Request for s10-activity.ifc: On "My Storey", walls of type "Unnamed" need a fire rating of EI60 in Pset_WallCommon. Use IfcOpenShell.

First a look at what the model holds.

```python
import ifcopenshell
import ifcopenshell.util.element

model = ifcopenshell.open("s10-activity.ifc")
print(model.schema)
storey = next(s for s in model.by_type("IfcBuildingStorey") if s.Name == "My Storey")
walls = [e for e in ifcopenshell.util.element.get_decomposition(storey) if e.is_a("IfcWall")]
seen = {}
for e in walls:
    element_type = ifcopenshell.util.element.get_type(e)
    key = (element_type.Name if element_type != e and element_type else None, ifcopenshell.util.element.get_pset(e, "Pset_WallCommon", "FireRating"))
    seen[key] = seen.get(key, 0) + 1
for (name, value), count in sorted(seen.items(), key=str):
    print(count, "x", name, "|", value)
```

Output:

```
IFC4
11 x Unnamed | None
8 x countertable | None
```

```python
import ifcopenshell
import ifcopenshell.api.pset
import ifcopenshell.util.element

model = ifcopenshell.open("s10-activity.ifc")

storey = next(s for s in model.by_type("IfcBuildingStorey") if s.Name == "My Storey")
walls = [e for e in ifcopenshell.util.element.get_decomposition(storey) if e.is_a("IfcWall")]

count = 0
for e in walls:
    element_type = ifcopenshell.util.element.get_type(e)
    if element_type in (None, e) or element_type.Name != "Unnamed":
        continue
    # add_pset returns the element's existing set when there is one.
    pset = ifcopenshell.api.pset.add_pset(model, product=e, name="Pset_WallCommon")
    ifcopenshell.api.pset.edit_pset(model, pset=pset, properties={"FireRating": "EI60"})
    count += 1

print(count, "walls updated")

model.write("s10-activity_edited.ifc")
```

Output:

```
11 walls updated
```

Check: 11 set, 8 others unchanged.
